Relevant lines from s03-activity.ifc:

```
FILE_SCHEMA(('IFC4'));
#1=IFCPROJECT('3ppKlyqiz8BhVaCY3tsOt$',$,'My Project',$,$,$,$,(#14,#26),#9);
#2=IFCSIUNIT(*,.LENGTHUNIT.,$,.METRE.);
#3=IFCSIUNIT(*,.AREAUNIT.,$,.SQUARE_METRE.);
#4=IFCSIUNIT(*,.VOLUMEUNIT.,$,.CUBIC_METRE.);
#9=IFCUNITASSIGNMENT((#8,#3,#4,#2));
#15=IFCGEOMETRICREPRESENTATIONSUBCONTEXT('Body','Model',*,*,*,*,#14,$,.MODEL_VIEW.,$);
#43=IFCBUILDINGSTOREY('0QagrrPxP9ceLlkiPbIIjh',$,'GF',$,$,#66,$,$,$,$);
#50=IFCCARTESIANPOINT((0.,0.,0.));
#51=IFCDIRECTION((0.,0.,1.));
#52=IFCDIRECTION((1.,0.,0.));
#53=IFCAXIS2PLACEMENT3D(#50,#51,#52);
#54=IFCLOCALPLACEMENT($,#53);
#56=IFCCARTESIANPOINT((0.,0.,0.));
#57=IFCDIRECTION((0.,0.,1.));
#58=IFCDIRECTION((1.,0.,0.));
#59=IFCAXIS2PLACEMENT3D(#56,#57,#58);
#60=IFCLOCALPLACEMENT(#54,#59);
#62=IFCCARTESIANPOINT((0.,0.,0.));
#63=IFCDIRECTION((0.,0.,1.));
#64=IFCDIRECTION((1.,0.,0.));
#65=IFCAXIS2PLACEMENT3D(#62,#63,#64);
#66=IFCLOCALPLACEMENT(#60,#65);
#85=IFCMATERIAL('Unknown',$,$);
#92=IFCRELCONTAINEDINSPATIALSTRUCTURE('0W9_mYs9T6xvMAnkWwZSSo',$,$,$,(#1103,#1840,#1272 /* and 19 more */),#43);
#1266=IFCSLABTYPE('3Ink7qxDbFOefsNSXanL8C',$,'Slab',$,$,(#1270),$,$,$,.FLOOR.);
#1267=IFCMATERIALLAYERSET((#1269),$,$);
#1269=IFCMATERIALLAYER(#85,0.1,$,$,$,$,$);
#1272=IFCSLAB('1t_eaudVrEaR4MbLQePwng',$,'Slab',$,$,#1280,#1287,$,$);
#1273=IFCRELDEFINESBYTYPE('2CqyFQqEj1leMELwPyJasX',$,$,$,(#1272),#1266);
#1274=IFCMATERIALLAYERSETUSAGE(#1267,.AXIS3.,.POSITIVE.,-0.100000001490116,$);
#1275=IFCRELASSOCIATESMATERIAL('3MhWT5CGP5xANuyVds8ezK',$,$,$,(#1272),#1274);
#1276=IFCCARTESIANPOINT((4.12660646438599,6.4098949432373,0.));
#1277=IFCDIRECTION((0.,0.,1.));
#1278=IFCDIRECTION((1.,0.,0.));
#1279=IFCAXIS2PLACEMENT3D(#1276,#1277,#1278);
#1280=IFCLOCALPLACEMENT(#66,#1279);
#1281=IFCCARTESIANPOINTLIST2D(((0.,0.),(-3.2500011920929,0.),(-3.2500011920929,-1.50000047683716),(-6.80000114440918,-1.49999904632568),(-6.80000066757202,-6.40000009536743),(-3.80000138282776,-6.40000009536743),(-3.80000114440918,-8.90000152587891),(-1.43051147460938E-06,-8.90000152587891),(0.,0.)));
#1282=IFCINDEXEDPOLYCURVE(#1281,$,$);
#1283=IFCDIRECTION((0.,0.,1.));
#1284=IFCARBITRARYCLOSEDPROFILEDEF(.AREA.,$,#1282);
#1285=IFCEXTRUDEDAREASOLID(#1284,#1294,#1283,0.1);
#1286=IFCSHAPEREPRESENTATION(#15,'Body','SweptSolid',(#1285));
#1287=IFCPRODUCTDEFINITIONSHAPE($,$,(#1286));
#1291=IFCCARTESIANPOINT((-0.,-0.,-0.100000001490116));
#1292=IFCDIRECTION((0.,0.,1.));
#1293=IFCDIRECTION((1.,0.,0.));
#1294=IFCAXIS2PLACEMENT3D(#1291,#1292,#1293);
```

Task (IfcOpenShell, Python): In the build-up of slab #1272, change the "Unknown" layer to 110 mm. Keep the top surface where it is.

```python
import ifcopenshell
import ifcopenshell.util.element
import ifcopenshell.util.representation

model = ifcopenshell.open("s03-activity.ifc")

layer_set = model.by_id(1267)
layer = next(l for l in layer_set.MaterialLayers if l.Material and l.Material.Name == "Unknown")
change = 0.11 - layer.LayerThickness
layer.LayerThickness += change

# Geometry does not follow the layer set by itself.
slabs = [e for e in ifcopenshell.util.element.get_elements_by_material(model, layer_set) if e.is_a("IfcSlab")]
for slab in sorted(slabs, key=lambda e: e.id()):
    body = ifcopenshell.util.representation.get_representation(slab, "Model", "Body")
    solid = body.Items[0]
    old_depth = solid.Depth
    solid.Depth += change
    # Extruded upwards: lower the start of the extrusion so the top stays.
    x, y, z = solid.Position.Location.Coordinates
    solid.Position.Location = model.createIfcCartesianPoint((x, y, z - change))
    print(slab.id(), f"{old_depth:g} -> {solid.Depth:g}")

# The layers are counted up from the underside, which has moved.
for usage in {ifcopenshell.util.element.get_material(slab) for slab in slabs}:
    usage.OffsetFromReferenceLine -= change

model.write("s03-activity_rev.ifc")
```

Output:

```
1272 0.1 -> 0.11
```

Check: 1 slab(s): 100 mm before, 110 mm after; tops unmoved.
